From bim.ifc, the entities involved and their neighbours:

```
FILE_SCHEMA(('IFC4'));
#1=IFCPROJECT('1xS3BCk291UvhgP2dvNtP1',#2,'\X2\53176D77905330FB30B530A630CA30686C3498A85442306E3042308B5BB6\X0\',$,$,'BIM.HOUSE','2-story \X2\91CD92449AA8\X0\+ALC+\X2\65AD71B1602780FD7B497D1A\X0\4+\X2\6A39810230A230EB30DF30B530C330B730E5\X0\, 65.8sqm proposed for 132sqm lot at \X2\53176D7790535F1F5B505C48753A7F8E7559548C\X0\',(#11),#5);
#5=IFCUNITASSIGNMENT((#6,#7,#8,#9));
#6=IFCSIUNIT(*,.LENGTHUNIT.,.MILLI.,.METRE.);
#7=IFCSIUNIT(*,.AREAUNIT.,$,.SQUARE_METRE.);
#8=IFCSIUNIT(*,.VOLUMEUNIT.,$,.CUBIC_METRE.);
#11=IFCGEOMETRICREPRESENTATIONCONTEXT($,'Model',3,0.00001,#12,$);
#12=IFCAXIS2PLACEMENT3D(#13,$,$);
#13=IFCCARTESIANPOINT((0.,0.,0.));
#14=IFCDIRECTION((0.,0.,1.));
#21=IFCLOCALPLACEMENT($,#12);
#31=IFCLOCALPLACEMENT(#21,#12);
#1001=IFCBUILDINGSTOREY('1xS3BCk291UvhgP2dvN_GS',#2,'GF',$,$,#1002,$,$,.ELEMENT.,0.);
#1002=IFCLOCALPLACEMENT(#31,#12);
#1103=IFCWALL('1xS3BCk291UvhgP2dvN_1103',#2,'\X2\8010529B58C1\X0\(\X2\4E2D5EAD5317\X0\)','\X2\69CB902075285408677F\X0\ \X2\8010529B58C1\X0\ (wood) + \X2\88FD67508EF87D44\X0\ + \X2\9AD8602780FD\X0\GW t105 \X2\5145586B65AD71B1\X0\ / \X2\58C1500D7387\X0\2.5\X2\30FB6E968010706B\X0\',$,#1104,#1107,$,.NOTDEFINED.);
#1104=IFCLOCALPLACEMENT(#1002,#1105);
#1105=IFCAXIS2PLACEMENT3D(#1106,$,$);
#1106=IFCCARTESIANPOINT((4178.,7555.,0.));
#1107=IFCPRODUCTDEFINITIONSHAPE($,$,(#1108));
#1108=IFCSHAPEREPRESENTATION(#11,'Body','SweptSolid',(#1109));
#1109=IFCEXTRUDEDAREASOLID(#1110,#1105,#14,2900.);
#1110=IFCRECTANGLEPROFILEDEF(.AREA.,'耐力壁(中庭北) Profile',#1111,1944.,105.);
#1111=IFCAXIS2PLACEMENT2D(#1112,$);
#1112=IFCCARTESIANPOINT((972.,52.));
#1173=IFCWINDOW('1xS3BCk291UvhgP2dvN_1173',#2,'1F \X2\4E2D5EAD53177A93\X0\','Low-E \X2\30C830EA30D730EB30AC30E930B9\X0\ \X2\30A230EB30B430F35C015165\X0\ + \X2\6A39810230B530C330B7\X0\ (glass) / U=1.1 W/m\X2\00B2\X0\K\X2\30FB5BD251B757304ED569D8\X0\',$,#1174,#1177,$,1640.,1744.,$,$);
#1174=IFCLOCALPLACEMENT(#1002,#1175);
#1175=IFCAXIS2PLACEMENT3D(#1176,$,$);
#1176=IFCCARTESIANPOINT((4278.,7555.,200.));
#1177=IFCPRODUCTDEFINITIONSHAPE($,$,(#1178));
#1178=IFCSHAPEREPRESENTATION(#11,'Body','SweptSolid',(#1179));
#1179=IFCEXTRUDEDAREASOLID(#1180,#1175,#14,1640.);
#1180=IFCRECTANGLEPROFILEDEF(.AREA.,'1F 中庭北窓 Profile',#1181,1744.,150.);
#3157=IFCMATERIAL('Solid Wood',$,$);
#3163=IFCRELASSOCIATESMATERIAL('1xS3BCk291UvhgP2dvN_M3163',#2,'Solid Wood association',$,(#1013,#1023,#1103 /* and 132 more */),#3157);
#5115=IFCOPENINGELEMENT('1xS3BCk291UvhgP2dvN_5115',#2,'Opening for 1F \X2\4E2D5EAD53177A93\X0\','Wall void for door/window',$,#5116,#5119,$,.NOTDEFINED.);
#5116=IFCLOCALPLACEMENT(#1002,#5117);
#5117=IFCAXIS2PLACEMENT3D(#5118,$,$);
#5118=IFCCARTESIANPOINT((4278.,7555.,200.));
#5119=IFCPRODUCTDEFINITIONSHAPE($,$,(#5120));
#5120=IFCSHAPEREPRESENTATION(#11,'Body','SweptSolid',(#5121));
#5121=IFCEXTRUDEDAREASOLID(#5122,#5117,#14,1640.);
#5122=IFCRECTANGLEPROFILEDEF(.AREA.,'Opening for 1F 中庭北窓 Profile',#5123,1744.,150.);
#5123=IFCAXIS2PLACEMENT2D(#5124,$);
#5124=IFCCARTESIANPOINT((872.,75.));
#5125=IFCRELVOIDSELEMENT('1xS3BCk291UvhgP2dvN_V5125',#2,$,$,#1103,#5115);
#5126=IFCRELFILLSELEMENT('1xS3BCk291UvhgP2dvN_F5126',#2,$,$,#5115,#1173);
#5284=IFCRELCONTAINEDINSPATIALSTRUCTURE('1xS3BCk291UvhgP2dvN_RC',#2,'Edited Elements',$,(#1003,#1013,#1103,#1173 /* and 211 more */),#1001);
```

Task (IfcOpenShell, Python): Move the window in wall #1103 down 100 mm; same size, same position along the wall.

```python
import numpy as np
import ifcopenshell
import ifcopenshell.api.geometry
import ifcopenshell.util.placement
import ifcopenshell.util.unit

model = ifcopenshell.open("bim.ifc")
unit_scale = ifcopenshell.util.unit.calculate_unit_scale(model)

window = model.by_id(1173)
opening = window.FillsVoids[0].RelatingOpeningElement
dz = -0.1 / unit_scale

shift = np.array([0.0, 0.0, dz])
# The window is not placed relative to its opening, so move both.
for product in (opening, window):
    matrix = ifcopenshell.util.placement.get_local_placement(product.ObjectPlacement)
    matrix[:3, 3] += shift
    ifcopenshell.api.geometry.edit_object_placement(model, product=product, matrix=matrix, is_si=False)

print(f"moved by {dz * unit_scale:+.3f} m")

model.write("bim_edited.ifc")
```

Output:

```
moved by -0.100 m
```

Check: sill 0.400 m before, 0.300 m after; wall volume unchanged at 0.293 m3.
